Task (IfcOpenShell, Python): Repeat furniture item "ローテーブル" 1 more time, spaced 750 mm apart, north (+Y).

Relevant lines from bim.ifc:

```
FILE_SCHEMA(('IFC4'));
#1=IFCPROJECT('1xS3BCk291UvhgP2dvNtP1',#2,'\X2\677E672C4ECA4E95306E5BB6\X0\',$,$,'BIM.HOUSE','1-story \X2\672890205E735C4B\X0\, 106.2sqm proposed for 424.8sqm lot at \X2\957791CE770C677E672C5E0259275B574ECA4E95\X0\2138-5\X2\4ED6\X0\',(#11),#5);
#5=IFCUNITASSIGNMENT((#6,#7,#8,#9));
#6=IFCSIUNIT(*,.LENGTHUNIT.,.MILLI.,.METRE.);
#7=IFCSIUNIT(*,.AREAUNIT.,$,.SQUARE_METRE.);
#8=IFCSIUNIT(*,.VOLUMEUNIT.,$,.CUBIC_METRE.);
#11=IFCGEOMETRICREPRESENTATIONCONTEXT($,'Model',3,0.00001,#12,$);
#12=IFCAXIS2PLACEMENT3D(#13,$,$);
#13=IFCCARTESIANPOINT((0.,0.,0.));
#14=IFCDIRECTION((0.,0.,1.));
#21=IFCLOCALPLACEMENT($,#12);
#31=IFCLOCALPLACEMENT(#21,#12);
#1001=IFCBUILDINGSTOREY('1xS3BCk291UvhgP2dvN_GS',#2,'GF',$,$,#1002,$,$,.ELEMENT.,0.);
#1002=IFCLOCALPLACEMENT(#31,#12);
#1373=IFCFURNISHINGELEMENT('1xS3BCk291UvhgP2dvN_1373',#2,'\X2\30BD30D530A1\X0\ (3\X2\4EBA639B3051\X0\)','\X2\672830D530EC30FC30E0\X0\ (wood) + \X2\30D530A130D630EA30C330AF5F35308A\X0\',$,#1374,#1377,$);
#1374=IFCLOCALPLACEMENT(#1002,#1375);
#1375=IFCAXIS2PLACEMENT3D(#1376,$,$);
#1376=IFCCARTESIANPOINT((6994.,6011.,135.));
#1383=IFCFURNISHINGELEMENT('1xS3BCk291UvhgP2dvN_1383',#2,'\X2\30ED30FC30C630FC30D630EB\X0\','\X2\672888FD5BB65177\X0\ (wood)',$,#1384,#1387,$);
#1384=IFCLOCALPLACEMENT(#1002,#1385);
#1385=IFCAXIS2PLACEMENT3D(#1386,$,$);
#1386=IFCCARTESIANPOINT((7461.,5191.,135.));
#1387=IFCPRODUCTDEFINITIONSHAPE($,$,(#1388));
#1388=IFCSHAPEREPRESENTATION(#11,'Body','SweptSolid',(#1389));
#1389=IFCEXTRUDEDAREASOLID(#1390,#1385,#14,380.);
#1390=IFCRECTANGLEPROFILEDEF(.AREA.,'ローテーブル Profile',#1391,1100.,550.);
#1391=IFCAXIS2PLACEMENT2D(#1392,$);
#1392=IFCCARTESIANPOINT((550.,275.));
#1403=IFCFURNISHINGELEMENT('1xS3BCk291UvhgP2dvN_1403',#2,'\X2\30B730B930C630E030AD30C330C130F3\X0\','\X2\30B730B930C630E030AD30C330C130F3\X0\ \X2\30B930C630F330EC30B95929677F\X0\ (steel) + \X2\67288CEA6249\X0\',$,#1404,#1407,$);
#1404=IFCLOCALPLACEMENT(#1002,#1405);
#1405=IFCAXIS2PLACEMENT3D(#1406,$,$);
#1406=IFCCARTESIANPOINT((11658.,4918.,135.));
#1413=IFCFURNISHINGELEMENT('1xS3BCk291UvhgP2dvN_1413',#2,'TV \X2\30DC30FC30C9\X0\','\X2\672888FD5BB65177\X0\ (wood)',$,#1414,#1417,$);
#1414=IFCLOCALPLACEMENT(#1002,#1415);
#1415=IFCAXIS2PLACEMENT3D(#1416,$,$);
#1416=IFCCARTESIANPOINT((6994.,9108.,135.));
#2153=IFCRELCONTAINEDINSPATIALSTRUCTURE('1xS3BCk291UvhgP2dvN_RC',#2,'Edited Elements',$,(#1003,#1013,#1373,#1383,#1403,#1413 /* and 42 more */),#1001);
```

```python
import numpy as np
import ifcopenshell
import ifcopenshell.api.geometry
import ifcopenshell.api.root
import ifcopenshell.util.element
import ifcopenshell.util.placement
import ifcopenshell.util.unit

model = ifcopenshell.open("bim.ifc")
unit_scale = ifcopenshell.util.unit.calculate_unit_scale(model)


def reuse_history(source, copy):
    """copy_class also copies each property set's owner history, people and application; keep the originals."""
    for rel in copy.IsDefinedBy:
        if rel.is_a("IfcRelDefinesByProperties") and (history := rel.RelatingPropertyDefinition.OwnerHistory):
            rel.RelatingPropertyDefinition.OwnerHistory = source.OwnerHistory
            ifcopenshell.util.element.remove_deep2(model, history)


source = model.by_id(1383)
base = ifcopenshell.util.placement.get_local_placement(source.ObjectPlacement)
step = np.array([0.0, 1.0, 0.0]) * 0.75 / unit_scale

for i in range(1, 2):
    copy = ifcopenshell.api.root.copy_class(model, product=source)
    copy.Representation = ifcopenshell.util.element.copy_deep(
        model, source.Representation, exclude=["IfcGeometricRepresentationContext", "IfcRepresentationMap"]
    )
    reuse_history(source, copy)
    matrix = base.copy()
    matrix[:3, 3] += i * step
    print("added at", matrix[:3, 3].round(3) + 0.0)
    ifcopenshell.api.geometry.edit_object_placement(model, product=copy, matrix=matrix, is_si=False)

model.write("bim_rev.ifc")
```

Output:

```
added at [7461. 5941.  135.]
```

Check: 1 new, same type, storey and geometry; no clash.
